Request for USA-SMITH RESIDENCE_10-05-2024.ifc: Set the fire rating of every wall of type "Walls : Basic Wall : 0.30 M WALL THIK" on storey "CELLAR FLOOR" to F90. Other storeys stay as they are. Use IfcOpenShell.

First a look at what the model holds.

```python
import ifcopenshell
import ifcopenshell.util.element

model = ifcopenshell.open("USA-SMITH RESIDENCE_10-05-2024.ifc")
print(model.schema)
storey = next(s for s in model.by_type("IfcBuildingStorey") if s.Name == "CELLAR FLOOR")
walls = [e for e in ifcopenshell.util.element.get_decomposition(storey) if e.is_a("IfcWall")]
seen = {}
for e in walls:
    element_type = ifcopenshell.util.element.get_type(e)
    key = (element_type.Name if element_type != e and element_type else None, ifcopenshell.util.element.get_pset(e, "Pset_WallCommon", "FireRating"))
    seen[key] = seen.get(key, 0) + 1
for (name, value), count in sorted(seen.items(), key=str):
    print(count, "x", name, "|", value)
```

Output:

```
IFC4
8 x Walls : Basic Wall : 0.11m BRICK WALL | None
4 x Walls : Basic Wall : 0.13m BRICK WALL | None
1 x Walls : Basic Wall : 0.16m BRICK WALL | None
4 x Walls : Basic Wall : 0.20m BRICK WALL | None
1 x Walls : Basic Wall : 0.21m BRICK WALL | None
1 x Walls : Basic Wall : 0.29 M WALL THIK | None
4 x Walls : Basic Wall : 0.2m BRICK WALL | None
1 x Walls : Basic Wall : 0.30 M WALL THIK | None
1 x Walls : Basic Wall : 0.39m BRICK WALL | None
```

```python
import ifcopenshell
import ifcopenshell.api.pset
import ifcopenshell.util.element

model = ifcopenshell.open("USA-SMITH RESIDENCE_10-05-2024.ifc")

storey = next(s for s in model.by_type("IfcBuildingStorey") if s.Name == "CELLAR FLOOR")
walls = [e for e in ifcopenshell.util.element.get_decomposition(storey) if e.is_a("IfcWall")]

count = 0
for e in walls:
    element_type = ifcopenshell.util.element.get_type(e)
    if element_type in (None, e) or element_type.Name != "Walls : Basic Wall : 0.30 M WALL THIK":
        continue
    # add_pset returns the element's existing set when there is one.
    pset = ifcopenshell.api.pset.add_pset(model, product=e, name="Pset_WallCommon")
    ifcopenshell.api.pset.edit_pset(model, pset=pset, properties={"FireRating": "F90"})
    count += 1

print(count, "walls updated")

model.write("USA-SMITH RESIDENCE_10-05-2024_v2.ifc")
```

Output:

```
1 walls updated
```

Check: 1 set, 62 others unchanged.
